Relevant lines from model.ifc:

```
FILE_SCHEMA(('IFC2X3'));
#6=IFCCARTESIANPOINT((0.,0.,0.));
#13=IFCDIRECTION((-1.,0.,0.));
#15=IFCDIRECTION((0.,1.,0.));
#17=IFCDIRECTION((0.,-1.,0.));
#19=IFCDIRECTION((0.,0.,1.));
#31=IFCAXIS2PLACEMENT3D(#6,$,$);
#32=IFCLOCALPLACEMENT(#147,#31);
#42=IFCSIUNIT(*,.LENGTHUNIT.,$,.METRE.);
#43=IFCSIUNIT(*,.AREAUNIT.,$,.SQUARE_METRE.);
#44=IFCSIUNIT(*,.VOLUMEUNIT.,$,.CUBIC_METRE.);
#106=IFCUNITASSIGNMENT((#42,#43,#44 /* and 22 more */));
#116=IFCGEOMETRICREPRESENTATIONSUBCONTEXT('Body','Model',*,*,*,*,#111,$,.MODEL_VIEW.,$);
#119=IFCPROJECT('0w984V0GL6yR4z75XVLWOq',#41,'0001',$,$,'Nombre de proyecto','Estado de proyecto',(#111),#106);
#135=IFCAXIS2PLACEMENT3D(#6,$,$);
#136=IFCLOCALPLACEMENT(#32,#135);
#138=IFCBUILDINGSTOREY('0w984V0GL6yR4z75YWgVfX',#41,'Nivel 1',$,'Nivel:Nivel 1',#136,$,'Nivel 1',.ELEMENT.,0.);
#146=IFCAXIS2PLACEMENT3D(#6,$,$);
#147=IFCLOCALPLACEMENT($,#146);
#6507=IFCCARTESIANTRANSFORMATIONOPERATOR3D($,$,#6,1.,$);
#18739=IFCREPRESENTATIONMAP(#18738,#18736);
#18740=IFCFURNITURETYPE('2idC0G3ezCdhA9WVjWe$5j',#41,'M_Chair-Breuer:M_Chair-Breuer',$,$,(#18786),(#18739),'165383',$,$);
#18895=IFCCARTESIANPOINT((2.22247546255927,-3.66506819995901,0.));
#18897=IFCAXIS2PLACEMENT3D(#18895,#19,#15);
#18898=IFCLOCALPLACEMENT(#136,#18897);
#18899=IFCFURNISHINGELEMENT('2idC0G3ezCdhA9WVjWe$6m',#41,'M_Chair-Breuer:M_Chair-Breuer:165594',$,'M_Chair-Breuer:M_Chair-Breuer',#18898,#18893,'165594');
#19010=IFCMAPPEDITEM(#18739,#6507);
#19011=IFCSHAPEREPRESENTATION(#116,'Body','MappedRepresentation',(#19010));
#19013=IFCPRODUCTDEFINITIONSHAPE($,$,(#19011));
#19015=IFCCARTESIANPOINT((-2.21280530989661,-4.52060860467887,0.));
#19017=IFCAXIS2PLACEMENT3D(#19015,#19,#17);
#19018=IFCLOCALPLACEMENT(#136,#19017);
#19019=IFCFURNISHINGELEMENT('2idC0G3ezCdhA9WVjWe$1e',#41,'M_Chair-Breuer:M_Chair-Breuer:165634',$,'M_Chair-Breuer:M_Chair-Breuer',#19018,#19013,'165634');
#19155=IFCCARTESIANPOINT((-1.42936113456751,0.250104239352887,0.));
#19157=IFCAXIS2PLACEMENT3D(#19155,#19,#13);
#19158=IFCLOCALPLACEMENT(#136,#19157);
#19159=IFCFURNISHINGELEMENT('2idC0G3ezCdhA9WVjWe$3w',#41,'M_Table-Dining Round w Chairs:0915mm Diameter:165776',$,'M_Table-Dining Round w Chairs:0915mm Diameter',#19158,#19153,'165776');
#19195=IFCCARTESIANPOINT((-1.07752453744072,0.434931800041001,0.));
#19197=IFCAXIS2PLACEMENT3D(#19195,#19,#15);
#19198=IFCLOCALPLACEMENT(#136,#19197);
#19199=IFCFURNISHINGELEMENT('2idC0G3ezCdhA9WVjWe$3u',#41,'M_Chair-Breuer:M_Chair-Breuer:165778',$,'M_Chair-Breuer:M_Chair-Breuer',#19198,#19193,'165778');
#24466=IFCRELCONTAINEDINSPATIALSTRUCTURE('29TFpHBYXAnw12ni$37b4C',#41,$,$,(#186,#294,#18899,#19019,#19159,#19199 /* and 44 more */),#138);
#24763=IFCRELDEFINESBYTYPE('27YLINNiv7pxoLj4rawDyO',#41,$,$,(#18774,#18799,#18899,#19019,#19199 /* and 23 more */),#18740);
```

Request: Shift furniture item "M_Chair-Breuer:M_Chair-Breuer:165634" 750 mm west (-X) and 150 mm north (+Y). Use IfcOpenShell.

```python
import ifcopenshell
import ifcopenshell.api.geometry
import ifcopenshell.util.placement
import ifcopenshell.util.unit

model = ifcopenshell.open("model.ifc")
unit_scale = ifcopenshell.util.unit.calculate_unit_scale(model)

item = model.by_guid("2idC0G3ezCdhA9WVjWe$1e")
matrix = ifcopenshell.util.placement.get_local_placement(item.ObjectPlacement)
matrix[0, 3] -= 0.75 / unit_scale
matrix[1, 3] += 0.15 / unit_scale
ifcopenshell.api.geometry.edit_object_placement(model, product=item, matrix=matrix, is_si=False)

print(ifcopenshell.util.placement.get_local_placement(item.ObjectPlacement).round(3) + 0.0)

model.write("model_v2.ifc")
```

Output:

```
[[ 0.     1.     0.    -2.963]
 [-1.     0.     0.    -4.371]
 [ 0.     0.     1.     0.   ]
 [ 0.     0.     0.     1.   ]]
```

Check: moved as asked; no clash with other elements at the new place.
